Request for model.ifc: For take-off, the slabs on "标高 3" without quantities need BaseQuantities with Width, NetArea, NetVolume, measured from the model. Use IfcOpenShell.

First a look at what the model holds.

```python
import ifcopenshell
import ifcopenshell.util.element
import ifcopenshell.util.unit

model = ifcopenshell.open("model.ifc")
print(model.schema)
for unit_type in ("LENGTHUNIT", "AREAUNIT", "VOLUMEUNIT"):
    print(unit_type, ifcopenshell.util.unit.calculate_unit_scale(model, unit_type))
storey = next(s for s in model.by_type("IfcBuildingStorey") if s.Name == "标高 3")
slabs = [e for e in ifcopenshell.util.element.get_decomposition(storey) if e.is_a("IfcSlab")]
for e in sorted(slabs, key=lambda e: e.id()):
    print(e.id(), e.is_a(), e.Name, list(ifcopenshell.util.element.get_psets(e, qtos_only=True)), sep=" | ")
```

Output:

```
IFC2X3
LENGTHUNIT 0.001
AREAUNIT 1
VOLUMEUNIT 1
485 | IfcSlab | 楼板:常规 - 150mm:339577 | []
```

```python
import ifcopenshell
import ifcopenshell.api.pset
import ifcopenshell.geom
import ifcopenshell.util.element
import ifcopenshell.util.shape
import ifcopenshell.util.unit

model = ifcopenshell.open("model.ifc")
unit_scale = ifcopenshell.util.unit.calculate_unit_scale(model)
area_scale = ifcopenshell.util.unit.calculate_unit_scale(model, "AREAUNIT")
volume_scale = ifcopenshell.util.unit.calculate_unit_scale(model, "VOLUMEUNIT")
settings = ifcopenshell.geom.settings()

storey = next(s for s in model.by_type("IfcBuildingStorey") if s.Name == "标高 3")
slabs = [e for e in ifcopenshell.util.element.get_decomposition(storey) if e.is_a("IfcSlab")]

for e in sorted(slabs, key=lambda e: e.id()):
    if ifcopenshell.util.element.get_psets(e, qtos_only=True, should_inherit=False):
        continue
    # Geometry comes back in metres, in the element's own axes.
    shape = ifcopenshell.geom.create_shape(settings, e)
    values = {
        "Width": ifcopenshell.util.shape.get_z(shape.geometry) / unit_scale,
        "NetArea": ifcopenshell.util.shape.get_footprint_area(shape.geometry) / area_scale,
        "NetVolume": ifcopenshell.util.shape.get_volume(shape.geometry) / volume_scale,
    }
    qto = ifcopenshell.api.pset.add_qto(model, product=e, name="BaseQuantities")
    ifcopenshell.api.pset.edit_qto(model, qto=qto, properties=values)
    print(e.id(), {k: round(v, 3) for k, v in values.items()})

model.write("model_edited.ifc")
```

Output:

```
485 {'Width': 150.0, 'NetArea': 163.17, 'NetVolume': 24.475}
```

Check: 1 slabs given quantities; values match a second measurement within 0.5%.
